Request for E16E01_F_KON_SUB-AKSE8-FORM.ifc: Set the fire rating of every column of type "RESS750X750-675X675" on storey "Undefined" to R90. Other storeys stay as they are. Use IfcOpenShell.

First a look at what the model holds.

```python
import ifcopenshell
import ifcopenshell.util.element

model = ifcopenshell.open("E16E01_F_KON_SUB-AKSE8-FORM.ifc")
print(model.schema)
storey = next(s for s in model.by_type("IfcBuildingStorey") if s.Name == "Undefined")
columns = [e for e in ifcopenshell.util.element.get_decomposition(storey) if e.is_a("IfcColumn")]
seen = {}
for e in columns:
    element_type = ifcopenshell.util.element.get_type(e)
    key = (element_type.Name if element_type != e and element_type else None, ifcopenshell.util.element.get_pset(e, "Pset_ColumnCommon", "FireRating"))
    seen[key] = seen.get(key, 0) + 1
for (name, value), count in sorted(seen.items(), key=str):
    print(count, "x", name, "|", value)
```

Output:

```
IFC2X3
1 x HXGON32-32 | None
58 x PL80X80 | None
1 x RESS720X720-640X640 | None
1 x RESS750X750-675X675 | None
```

```python
import ifcopenshell
import ifcopenshell.api.pset
import ifcopenshell.util.element

model = ifcopenshell.open("E16E01_F_KON_SUB-AKSE8-FORM.ifc")

storey = next(s for s in model.by_type("IfcBuildingStorey") if s.Name == "Undefined")
columns = [e for e in ifcopenshell.util.element.get_decomposition(storey) if e.is_a("IfcColumn")]

count = 0
for e in columns:
    element_type = ifcopenshell.util.element.get_type(e)
    if element_type in (None, e) or element_type.Name != "RESS750X750-675X675":
        continue
    # add_pset returns the element's existing set when there is one.
    pset = ifcopenshell.api.pset.add_pset(model, product=e, name="Pset_ColumnCommon")
    ifcopenshell.api.pset.edit_pset(model, pset=pset, properties={"FireRating": "R90"})
    count += 1

print(count, "columns updated")

model.write("E16E01_F_KON_SUB-AKSE8-FORM_edited.ifc")
```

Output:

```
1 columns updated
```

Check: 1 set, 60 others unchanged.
